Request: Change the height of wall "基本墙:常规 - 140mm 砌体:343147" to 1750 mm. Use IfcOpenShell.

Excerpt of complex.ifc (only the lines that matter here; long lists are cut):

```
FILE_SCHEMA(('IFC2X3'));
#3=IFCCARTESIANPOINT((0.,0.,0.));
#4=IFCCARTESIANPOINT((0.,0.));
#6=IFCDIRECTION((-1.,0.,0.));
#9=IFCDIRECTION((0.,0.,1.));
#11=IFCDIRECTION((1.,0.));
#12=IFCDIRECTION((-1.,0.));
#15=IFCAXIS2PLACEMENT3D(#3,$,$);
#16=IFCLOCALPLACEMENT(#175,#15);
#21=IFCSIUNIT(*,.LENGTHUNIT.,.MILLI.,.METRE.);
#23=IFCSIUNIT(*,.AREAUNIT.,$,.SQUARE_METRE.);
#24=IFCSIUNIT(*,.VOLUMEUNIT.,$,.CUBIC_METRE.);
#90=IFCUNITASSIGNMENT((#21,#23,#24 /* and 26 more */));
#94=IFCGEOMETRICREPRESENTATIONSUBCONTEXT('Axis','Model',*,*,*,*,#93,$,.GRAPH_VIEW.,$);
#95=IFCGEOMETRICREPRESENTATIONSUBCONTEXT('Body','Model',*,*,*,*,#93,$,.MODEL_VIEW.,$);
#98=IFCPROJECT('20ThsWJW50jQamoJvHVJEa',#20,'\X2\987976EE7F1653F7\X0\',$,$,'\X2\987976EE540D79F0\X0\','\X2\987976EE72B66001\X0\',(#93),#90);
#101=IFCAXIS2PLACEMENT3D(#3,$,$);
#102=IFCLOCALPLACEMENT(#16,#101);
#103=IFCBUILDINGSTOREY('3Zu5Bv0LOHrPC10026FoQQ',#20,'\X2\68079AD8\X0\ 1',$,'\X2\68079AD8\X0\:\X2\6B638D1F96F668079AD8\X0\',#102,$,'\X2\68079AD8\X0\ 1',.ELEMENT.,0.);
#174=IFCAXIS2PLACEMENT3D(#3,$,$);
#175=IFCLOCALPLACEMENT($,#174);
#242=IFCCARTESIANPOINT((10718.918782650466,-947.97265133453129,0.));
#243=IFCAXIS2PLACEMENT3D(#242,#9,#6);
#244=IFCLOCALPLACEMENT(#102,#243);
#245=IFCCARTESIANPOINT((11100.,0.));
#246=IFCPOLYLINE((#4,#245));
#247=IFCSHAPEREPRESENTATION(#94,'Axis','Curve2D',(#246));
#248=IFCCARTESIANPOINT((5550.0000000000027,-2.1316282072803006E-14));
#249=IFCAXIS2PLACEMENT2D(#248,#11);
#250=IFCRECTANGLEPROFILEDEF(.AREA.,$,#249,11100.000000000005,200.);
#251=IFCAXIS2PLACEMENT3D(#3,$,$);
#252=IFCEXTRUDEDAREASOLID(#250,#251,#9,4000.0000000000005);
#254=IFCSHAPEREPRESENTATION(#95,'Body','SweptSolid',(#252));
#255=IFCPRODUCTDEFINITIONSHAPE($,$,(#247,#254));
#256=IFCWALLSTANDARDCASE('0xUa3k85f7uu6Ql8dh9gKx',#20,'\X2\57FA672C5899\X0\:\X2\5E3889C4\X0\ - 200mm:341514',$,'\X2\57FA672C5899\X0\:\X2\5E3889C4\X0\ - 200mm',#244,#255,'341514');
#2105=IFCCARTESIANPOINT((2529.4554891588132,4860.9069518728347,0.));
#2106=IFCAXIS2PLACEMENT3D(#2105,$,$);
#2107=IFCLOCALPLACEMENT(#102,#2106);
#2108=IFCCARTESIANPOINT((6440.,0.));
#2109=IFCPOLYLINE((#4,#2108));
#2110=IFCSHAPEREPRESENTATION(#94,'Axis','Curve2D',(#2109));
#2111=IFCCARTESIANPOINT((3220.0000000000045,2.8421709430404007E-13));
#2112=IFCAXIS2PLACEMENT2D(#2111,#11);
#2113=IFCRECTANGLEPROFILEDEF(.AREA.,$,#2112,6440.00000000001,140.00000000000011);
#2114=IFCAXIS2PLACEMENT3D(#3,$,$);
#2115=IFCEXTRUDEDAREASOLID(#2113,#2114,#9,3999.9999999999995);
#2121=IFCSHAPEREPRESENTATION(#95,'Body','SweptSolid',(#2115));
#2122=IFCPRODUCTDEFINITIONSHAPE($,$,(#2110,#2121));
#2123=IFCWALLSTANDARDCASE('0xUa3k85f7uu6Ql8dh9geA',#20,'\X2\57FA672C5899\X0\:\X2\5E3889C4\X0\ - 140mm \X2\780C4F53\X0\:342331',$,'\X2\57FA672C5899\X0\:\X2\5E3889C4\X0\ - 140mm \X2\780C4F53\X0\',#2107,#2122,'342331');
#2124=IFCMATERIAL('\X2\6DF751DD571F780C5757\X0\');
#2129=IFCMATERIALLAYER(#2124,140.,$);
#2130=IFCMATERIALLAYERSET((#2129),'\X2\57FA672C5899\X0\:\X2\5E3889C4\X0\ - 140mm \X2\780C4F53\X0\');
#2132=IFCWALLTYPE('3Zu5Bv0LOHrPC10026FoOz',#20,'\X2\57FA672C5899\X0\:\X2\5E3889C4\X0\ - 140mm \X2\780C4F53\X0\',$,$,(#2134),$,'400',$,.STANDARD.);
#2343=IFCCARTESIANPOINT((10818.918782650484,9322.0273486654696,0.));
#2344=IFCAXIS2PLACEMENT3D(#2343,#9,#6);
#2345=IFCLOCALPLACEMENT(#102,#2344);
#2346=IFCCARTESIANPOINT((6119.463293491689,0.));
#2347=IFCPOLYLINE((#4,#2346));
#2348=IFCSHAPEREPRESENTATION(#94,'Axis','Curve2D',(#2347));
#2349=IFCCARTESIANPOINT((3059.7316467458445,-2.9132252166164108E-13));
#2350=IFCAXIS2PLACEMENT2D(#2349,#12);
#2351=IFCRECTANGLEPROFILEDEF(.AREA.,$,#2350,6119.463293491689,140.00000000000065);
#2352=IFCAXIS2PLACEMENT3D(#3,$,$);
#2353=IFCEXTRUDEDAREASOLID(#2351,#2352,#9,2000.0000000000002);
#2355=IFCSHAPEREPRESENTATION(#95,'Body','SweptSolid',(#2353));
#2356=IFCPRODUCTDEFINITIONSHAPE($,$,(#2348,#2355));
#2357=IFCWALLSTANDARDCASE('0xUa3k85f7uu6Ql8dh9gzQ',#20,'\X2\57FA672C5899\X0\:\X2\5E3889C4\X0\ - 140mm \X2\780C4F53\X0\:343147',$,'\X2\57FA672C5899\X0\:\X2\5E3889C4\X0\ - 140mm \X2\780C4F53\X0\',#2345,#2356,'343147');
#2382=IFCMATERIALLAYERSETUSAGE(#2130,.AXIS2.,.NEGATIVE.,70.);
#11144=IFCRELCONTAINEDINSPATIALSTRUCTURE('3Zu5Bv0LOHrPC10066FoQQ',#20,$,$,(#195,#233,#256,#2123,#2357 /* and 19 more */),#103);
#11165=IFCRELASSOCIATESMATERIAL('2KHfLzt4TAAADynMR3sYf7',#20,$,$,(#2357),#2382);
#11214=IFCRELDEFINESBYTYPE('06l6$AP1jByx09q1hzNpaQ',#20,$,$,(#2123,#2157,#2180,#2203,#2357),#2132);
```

```python
import ifcopenshell
import ifcopenshell.geom
import ifcopenshell.util.representation
import ifcopenshell.util.shape

model = ifcopenshell.open("complex.ifc")
settings = ifcopenshell.geom.settings()


def volume(element):
    """Net volume in cubic metres, openings subtracted."""
    shape = ifcopenshell.geom.create_shape(settings, element)
    return ifcopenshell.util.shape.get_volume(shape.geometry)


wall = model.by_guid("0xUa3k85f7uu6Ql8dh9gzQ")
before = volume(wall)

body = ifcopenshell.util.representation.get_representation(wall, "Model", "Body")
solid = body.Items[0]
old_height = solid.Depth
solid.Depth = 1750.0
after = volume(wall)

print(f"height {old_height:g} -> {solid.Depth:g}, volume {before:.3f} -> {after:.3f} m3")

model.write("complex_rev.ifc")
```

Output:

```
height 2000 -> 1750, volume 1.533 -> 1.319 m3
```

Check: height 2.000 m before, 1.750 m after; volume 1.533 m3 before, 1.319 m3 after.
